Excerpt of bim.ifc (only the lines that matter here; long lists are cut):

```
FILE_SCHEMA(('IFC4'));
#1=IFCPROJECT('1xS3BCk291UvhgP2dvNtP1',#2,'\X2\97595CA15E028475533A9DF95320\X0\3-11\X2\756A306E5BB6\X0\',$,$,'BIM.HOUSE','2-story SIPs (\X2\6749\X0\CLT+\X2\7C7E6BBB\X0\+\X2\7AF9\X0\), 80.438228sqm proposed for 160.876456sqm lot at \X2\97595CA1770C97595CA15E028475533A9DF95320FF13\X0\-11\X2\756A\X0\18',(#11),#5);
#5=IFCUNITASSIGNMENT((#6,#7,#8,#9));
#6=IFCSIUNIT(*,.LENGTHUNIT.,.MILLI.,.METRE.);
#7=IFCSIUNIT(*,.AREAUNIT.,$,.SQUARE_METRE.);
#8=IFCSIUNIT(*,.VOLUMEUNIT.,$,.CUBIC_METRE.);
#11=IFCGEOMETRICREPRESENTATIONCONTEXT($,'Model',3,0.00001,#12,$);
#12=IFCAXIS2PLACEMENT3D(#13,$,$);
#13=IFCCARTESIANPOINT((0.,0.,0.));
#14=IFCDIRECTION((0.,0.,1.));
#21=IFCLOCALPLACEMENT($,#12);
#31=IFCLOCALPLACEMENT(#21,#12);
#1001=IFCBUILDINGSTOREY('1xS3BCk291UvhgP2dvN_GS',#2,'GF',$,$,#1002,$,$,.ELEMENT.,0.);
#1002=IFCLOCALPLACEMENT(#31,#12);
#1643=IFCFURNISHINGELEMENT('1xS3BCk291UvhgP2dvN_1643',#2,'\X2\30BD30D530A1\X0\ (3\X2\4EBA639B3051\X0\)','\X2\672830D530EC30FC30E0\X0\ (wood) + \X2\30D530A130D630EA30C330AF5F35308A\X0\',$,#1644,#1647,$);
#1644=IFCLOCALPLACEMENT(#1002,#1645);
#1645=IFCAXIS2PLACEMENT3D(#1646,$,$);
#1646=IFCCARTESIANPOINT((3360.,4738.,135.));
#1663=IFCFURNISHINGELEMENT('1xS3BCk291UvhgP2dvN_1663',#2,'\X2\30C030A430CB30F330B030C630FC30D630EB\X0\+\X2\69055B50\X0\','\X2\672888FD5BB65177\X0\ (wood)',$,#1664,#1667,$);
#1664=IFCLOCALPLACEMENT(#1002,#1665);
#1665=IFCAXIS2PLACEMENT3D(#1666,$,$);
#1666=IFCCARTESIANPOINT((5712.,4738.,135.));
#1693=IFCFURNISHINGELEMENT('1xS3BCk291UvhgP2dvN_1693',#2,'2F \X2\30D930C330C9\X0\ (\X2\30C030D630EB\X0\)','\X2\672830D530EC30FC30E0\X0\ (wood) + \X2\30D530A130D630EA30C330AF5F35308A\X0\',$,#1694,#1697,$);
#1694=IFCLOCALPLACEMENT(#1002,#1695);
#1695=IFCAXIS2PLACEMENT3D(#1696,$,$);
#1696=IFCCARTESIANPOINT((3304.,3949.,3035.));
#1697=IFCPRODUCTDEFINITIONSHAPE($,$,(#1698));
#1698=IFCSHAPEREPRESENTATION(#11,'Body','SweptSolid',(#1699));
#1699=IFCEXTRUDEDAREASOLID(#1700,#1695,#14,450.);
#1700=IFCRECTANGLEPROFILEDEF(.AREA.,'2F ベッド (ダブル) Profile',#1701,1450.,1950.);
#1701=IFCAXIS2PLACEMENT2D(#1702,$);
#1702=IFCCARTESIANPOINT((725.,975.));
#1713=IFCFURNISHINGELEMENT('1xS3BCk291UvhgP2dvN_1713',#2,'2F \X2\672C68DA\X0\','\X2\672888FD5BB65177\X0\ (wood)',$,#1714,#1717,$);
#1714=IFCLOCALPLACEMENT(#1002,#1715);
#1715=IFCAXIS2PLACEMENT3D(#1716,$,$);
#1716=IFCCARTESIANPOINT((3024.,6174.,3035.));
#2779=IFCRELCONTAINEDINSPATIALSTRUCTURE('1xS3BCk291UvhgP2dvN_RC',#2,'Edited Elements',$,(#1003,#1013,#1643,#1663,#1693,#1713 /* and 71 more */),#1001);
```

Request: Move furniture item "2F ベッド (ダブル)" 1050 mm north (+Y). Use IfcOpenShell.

```python
import ifcopenshell
import ifcopenshell.api.geometry
import ifcopenshell.util.placement
import ifcopenshell.util.unit

model = ifcopenshell.open("bim.ifc")
unit_scale = ifcopenshell.util.unit.calculate_unit_scale(model)

item = model.by_id(1693)
matrix = ifcopenshell.util.placement.get_local_placement(item.ObjectPlacement)
matrix[1, 3] += 1.05 / unit_scale
ifcopenshell.api.geometry.edit_object_placement(model, product=item, matrix=matrix, is_si=False)

print(ifcopenshell.util.placement.get_local_placement(item.ObjectPlacement).round(3) + 0.0)

model.write("bim_v2.ifc")
```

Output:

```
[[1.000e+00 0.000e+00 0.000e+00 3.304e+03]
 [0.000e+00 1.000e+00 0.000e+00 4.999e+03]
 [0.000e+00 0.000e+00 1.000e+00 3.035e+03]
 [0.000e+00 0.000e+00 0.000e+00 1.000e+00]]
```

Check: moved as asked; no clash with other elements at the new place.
